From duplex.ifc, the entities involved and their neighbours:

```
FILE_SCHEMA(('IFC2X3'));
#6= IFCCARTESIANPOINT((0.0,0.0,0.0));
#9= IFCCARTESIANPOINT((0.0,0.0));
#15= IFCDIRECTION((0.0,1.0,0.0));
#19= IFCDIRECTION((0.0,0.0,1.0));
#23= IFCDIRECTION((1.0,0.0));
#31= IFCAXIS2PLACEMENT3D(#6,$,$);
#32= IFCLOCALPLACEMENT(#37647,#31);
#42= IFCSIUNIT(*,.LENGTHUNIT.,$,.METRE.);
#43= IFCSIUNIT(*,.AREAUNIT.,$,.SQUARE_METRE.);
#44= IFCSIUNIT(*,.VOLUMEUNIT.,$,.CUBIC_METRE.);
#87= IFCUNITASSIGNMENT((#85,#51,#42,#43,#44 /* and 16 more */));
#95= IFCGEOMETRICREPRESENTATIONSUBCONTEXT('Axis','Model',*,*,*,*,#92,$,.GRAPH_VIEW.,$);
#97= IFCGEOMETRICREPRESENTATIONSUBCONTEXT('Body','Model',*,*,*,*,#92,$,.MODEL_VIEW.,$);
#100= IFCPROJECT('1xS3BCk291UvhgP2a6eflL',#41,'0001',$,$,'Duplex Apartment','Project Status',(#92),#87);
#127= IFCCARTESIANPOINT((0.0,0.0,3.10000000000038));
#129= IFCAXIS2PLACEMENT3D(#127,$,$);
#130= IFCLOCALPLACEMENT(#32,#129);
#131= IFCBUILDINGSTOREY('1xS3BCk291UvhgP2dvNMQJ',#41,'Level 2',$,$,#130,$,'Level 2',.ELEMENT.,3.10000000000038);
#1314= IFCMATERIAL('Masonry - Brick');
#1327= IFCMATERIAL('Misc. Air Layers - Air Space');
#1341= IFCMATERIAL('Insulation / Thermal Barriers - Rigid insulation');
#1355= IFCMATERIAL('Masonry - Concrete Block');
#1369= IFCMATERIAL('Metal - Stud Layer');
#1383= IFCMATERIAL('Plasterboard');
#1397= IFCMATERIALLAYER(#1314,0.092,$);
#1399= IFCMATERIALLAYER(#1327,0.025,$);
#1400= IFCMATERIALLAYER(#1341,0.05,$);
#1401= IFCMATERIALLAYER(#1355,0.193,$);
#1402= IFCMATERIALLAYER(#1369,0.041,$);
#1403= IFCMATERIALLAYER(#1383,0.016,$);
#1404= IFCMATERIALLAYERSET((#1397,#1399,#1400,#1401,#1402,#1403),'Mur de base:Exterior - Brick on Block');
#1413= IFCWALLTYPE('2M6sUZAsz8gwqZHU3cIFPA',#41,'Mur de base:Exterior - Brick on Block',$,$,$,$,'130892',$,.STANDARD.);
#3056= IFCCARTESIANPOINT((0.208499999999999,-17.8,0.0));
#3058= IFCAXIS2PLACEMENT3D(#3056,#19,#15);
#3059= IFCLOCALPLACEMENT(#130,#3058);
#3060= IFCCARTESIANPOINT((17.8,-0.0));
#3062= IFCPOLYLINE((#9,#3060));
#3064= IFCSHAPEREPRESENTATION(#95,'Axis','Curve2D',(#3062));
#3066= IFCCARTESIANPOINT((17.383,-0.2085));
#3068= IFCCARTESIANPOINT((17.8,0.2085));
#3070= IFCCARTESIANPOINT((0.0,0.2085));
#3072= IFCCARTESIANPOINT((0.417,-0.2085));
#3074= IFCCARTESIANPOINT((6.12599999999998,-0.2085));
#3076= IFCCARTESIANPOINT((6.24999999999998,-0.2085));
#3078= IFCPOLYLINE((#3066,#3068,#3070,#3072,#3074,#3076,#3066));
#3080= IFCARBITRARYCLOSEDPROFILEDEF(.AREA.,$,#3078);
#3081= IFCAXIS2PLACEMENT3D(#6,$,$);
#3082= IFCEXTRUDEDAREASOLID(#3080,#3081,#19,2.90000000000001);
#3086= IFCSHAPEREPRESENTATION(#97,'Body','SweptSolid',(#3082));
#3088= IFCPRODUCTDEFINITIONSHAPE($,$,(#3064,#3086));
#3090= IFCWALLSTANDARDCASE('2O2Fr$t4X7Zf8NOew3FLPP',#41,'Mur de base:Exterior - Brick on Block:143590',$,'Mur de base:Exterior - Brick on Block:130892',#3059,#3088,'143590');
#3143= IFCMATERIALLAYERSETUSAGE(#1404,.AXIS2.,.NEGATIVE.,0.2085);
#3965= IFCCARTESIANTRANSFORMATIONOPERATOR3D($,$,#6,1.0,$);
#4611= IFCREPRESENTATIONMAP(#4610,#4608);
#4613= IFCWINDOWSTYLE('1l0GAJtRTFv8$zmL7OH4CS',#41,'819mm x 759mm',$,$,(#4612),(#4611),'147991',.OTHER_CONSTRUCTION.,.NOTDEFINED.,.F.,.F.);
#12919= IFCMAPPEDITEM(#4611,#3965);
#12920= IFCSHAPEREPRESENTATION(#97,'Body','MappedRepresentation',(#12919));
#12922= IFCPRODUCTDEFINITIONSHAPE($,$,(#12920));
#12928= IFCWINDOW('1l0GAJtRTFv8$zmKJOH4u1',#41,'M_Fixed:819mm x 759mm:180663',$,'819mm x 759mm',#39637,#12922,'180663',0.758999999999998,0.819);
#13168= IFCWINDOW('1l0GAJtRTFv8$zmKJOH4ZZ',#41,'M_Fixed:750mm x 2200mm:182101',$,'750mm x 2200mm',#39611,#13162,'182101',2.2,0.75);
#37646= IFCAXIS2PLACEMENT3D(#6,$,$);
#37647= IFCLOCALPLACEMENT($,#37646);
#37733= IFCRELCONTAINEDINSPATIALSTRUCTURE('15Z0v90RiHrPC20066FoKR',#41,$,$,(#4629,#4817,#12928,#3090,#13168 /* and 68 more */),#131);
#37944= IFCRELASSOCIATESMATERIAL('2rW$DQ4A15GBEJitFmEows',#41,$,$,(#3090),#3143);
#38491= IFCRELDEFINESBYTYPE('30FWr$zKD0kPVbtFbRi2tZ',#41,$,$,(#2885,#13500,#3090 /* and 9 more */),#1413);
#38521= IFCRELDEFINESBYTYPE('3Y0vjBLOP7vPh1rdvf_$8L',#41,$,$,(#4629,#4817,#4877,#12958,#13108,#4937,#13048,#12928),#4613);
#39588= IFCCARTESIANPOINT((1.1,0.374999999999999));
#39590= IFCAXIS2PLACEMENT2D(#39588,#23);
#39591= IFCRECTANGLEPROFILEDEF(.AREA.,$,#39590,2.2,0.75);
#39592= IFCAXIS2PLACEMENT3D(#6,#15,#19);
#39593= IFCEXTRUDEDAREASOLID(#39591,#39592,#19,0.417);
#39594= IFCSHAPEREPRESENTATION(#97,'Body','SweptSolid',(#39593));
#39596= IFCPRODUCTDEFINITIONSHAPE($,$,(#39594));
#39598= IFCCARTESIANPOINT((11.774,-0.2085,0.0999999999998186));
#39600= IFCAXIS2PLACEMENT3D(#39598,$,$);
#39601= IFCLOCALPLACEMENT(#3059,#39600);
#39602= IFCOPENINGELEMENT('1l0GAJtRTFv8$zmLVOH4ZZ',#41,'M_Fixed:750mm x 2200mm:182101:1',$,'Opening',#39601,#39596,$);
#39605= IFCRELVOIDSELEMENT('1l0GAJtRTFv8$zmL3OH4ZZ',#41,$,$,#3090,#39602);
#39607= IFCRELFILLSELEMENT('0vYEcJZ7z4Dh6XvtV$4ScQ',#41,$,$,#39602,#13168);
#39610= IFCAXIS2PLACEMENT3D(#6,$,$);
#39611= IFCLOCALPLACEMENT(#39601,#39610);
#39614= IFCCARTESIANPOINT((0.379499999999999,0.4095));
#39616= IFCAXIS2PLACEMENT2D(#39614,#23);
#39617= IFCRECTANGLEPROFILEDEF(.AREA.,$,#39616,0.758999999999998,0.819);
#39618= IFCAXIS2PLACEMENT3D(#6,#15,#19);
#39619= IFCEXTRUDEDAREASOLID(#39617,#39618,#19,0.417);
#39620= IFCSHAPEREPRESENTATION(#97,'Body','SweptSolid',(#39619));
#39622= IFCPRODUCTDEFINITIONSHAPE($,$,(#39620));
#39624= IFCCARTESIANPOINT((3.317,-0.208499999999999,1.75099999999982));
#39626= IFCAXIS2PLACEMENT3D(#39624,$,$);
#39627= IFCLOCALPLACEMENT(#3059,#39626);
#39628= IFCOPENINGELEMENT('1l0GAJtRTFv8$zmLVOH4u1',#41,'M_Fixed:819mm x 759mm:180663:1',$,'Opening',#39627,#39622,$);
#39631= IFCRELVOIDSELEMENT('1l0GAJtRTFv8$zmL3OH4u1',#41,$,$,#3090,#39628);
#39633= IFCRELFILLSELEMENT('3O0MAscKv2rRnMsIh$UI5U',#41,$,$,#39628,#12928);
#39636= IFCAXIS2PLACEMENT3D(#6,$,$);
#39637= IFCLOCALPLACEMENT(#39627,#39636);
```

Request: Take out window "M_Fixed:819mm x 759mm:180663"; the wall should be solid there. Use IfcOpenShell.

```python
import ifcopenshell
import ifcopenshell.api.feature
import ifcopenshell.api.root
import ifcopenshell.geom
import ifcopenshell.util.shape

model = ifcopenshell.open("duplex.ifc")
settings = ifcopenshell.geom.settings()


def volume(element):
    """Net volume in cubic metres, openings subtracted."""
    shape = ifcopenshell.geom.create_shape(settings, element)
    return ifcopenshell.util.shape.get_volume(shape.geometry)


window = model.by_guid("1l0GAJtRTFv8$zmKJOH4u1")
opening = window.FillsVoids[0].RelatingOpeningElement
wall = opening.VoidsElements[0].RelatingBuildingElement
before = volume(wall)

ifcopenshell.api.root.remove_product(model, product=window)
ifcopenshell.api.feature.remove_feature(model, feature=opening)

after = volume(wall)

print(f"wall volume {before:.3f} -> {after:.3f} m3")

model.write("duplex_updated.ifc")
```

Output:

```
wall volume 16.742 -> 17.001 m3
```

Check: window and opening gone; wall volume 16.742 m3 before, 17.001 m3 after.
